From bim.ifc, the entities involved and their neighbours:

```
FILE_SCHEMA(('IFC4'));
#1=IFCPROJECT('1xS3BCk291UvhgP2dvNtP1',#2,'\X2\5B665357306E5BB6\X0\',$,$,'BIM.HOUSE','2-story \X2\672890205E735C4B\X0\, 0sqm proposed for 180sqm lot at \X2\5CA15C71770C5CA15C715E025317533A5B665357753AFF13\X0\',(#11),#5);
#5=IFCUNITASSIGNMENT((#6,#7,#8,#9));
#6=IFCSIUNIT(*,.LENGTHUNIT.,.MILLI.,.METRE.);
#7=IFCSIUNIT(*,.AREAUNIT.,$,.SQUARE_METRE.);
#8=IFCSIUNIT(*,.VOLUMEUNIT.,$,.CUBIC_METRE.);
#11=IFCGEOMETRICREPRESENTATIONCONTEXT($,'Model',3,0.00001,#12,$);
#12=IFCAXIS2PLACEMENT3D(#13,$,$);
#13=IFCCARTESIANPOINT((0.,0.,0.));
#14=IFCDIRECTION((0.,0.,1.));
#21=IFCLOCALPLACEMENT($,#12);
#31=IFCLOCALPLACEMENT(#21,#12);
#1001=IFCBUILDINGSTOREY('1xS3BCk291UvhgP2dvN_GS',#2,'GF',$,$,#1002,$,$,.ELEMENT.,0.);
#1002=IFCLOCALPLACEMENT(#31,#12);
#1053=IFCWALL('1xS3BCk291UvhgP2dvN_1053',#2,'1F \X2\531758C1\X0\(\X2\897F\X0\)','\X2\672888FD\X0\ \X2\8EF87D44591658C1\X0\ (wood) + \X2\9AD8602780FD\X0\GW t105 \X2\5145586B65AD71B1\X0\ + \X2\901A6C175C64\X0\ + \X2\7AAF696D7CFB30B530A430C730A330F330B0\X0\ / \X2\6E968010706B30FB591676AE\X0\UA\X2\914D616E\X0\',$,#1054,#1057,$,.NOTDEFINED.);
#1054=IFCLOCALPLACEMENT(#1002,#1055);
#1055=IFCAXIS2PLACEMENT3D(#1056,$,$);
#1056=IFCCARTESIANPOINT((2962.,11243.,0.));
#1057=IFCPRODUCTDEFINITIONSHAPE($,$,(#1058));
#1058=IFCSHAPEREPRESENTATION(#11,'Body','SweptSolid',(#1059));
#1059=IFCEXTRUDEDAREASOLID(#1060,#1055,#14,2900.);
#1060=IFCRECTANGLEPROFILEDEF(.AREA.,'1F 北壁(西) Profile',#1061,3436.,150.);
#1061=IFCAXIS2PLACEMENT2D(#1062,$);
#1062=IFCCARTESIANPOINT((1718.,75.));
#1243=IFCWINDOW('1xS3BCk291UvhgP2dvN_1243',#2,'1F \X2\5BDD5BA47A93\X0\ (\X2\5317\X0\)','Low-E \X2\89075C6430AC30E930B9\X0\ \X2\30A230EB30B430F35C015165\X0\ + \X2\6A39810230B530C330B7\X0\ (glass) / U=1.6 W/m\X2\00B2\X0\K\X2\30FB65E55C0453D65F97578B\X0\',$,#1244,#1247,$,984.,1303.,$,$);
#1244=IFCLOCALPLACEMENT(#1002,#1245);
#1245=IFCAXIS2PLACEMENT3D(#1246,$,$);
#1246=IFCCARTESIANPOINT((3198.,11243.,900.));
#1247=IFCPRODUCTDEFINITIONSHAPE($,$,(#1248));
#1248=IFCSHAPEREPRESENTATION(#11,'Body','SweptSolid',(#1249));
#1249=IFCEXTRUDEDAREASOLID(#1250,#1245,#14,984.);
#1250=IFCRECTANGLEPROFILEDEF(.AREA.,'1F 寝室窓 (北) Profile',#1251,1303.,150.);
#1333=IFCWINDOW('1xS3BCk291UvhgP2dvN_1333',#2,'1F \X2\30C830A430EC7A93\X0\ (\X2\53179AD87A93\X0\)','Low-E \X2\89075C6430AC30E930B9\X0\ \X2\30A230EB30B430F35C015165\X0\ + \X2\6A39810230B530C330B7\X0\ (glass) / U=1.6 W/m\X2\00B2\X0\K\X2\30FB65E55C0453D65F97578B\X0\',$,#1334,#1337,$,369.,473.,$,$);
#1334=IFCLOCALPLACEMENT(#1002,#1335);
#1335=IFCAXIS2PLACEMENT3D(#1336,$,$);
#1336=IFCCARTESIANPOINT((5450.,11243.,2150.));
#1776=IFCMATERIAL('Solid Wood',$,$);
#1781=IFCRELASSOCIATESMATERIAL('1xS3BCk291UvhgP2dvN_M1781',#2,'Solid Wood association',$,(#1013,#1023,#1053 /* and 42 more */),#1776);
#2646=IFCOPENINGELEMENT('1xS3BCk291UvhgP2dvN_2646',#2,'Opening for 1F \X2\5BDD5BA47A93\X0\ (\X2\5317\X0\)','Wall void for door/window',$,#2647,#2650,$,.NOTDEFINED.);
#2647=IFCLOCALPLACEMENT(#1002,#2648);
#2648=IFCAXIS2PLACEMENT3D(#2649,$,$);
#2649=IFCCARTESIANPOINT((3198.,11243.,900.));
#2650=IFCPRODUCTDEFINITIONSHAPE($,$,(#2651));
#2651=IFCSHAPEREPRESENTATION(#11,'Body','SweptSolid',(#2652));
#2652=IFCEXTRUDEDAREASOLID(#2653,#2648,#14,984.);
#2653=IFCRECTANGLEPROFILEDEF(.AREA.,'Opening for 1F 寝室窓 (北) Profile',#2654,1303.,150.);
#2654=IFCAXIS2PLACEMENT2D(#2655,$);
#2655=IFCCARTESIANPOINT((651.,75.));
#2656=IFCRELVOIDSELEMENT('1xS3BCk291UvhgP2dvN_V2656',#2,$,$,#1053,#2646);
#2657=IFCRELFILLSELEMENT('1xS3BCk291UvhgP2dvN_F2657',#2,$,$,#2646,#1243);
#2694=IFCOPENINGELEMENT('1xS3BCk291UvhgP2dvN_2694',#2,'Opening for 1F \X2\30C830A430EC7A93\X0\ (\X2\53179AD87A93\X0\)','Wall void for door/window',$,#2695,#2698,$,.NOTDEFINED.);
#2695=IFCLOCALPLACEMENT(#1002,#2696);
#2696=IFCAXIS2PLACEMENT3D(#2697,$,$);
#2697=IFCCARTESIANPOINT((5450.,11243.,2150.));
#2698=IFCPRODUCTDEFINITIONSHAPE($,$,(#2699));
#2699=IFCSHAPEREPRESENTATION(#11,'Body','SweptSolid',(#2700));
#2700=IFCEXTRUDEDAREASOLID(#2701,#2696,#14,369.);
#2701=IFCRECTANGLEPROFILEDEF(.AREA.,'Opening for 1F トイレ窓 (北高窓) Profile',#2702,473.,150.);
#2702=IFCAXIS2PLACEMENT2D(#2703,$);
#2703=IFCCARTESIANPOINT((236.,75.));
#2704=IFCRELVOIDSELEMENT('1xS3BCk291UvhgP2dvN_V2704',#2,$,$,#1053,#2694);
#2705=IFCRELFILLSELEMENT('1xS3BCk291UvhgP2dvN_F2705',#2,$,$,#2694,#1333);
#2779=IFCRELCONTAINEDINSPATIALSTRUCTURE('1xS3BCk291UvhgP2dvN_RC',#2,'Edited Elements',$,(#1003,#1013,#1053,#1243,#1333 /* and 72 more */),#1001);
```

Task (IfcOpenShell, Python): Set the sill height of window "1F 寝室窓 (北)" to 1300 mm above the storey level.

```python
import numpy as np
import ifcopenshell
import ifcopenshell.api.geometry
import ifcopenshell.geom
import ifcopenshell.util.element
import ifcopenshell.util.placement
import ifcopenshell.util.shape
import ifcopenshell.util.unit

model = ifcopenshell.open("bim.ifc")
unit_scale = ifcopenshell.util.unit.calculate_unit_scale(model)

window = model.by_guid("1xS3BCk291UvhgP2dvN_1243")
opening = window.FillsVoids[0].RelatingOpeningElement
storey = ifcopenshell.util.element.get_container(window, ifc_class="IfcBuildingStorey")
level = ifcopenshell.util.placement.get_local_placement(storey.ObjectPlacement)[2, 3]

# The opening's origin need not be at the sill, so measure its lowest point.
shape = ifcopenshell.geom.create_shape(ifcopenshell.geom.settings(), opening)
bottom = ifcopenshell.util.shape.get_shape_bottom_elevation(shape, shape.geometry) / unit_scale
dz = level + 1300.0 - bottom

shift = np.array([0.0, 0.0, dz])
# The window is not placed relative to its opening, so move both.
for product in (opening, window):
    matrix = ifcopenshell.util.placement.get_local_placement(product.ObjectPlacement)
    matrix[:3, 3] += shift
    ifcopenshell.api.geometry.edit_object_placement(model, product=product, matrix=matrix, is_si=False)

print(f"moved by {dz * unit_scale:+.3f} m")

model.write("bim_updated.ifc")
```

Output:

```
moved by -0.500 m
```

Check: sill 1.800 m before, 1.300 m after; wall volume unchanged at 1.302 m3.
